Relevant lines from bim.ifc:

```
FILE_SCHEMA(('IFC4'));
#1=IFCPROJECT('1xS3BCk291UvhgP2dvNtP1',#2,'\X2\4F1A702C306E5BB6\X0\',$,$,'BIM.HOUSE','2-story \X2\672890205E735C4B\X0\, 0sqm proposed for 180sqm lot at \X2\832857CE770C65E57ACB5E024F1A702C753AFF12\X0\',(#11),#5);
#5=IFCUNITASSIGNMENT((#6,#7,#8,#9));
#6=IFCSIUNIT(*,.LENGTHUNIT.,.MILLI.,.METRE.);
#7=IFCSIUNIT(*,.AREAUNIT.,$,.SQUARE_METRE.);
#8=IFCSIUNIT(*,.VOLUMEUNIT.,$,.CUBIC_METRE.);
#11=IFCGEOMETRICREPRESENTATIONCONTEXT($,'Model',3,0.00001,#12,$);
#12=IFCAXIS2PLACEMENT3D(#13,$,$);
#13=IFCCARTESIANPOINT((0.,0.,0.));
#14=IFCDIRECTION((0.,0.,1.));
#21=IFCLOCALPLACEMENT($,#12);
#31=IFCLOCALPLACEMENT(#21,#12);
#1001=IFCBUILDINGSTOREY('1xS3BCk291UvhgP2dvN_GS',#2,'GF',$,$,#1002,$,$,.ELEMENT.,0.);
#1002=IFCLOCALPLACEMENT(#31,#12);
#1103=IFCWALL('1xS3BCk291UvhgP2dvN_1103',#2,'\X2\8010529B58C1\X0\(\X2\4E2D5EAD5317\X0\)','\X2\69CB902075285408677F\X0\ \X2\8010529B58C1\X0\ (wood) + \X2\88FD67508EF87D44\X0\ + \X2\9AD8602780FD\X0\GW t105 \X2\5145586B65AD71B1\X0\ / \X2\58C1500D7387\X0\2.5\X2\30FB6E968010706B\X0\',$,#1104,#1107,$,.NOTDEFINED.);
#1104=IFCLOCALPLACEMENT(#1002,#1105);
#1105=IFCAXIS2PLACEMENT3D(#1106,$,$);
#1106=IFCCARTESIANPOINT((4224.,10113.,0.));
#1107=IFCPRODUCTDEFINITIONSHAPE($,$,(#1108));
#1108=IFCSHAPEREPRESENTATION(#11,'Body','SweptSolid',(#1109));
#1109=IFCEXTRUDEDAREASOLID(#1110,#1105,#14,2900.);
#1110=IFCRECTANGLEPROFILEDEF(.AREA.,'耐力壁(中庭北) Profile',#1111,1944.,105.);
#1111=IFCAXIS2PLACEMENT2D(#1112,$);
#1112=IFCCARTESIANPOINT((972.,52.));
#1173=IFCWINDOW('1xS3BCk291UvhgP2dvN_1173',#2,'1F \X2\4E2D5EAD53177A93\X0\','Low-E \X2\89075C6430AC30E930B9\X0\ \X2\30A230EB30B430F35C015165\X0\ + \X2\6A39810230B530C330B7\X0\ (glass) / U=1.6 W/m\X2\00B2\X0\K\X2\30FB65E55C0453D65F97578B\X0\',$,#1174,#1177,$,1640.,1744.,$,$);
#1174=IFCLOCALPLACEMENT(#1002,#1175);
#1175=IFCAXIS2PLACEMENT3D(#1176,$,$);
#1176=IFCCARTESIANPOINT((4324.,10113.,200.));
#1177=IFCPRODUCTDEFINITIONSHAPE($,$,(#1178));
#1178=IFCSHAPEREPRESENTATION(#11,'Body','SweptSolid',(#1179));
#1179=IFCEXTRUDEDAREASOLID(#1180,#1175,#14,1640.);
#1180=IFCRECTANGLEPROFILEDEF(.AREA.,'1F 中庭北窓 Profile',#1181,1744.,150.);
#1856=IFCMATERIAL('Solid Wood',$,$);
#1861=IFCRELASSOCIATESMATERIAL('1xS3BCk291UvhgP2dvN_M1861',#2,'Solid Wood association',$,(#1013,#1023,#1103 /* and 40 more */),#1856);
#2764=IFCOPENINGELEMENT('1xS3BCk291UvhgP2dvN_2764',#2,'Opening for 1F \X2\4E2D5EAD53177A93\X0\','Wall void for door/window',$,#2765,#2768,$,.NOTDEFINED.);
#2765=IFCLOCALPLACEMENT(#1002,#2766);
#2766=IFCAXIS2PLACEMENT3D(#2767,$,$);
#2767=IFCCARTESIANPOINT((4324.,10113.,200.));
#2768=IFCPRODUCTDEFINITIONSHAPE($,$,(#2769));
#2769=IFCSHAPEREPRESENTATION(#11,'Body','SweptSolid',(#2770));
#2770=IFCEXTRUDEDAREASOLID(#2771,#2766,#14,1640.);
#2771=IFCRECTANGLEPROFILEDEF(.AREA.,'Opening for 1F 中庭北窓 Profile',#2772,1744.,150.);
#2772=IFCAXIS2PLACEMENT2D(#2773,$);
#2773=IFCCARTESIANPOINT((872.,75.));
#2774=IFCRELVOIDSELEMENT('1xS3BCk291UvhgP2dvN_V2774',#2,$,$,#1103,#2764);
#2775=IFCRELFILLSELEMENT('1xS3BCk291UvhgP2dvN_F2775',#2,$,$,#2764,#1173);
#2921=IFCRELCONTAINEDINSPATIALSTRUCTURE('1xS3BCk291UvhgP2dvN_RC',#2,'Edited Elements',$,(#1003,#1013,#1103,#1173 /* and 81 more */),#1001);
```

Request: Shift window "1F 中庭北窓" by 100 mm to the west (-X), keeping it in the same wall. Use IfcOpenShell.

```python
import ifcopenshell
import ifcopenshell.api.geometry
import ifcopenshell.util.placement
import ifcopenshell.util.unit

model = ifcopenshell.open("bim.ifc")
unit_scale = ifcopenshell.util.unit.calculate_unit_scale(model)

window = model.by_guid("1xS3BCk291UvhgP2dvN_1173")
opening = window.FillsVoids[0].RelatingOpeningElement
wall = opening.VoidsElements[0].RelatingBuildingElement

wall_matrix = ifcopenshell.util.placement.get_local_placement(wall.ObjectPlacement)
shift = wall_matrix[:3, 0] * -0.1 / unit_scale
before = ifcopenshell.util.placement.get_local_placement(window.ObjectPlacement)[:3, 3].copy()

# The window is not placed relative to its opening, so move both.
for product in (opening, window):
    matrix = ifcopenshell.util.placement.get_local_placement(product.ObjectPlacement)
    matrix[:3, 3] += shift
    ifcopenshell.api.geometry.edit_object_placement(model, product=product, matrix=matrix, is_si=False)

after = ifcopenshell.util.placement.get_local_placement(window.ObjectPlacement)[:3, 3]
print("window moved by", (after - before).round(3) + 0.0)

model.write("bim_v2.ifc")
```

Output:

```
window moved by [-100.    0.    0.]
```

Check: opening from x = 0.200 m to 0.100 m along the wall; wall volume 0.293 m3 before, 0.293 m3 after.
